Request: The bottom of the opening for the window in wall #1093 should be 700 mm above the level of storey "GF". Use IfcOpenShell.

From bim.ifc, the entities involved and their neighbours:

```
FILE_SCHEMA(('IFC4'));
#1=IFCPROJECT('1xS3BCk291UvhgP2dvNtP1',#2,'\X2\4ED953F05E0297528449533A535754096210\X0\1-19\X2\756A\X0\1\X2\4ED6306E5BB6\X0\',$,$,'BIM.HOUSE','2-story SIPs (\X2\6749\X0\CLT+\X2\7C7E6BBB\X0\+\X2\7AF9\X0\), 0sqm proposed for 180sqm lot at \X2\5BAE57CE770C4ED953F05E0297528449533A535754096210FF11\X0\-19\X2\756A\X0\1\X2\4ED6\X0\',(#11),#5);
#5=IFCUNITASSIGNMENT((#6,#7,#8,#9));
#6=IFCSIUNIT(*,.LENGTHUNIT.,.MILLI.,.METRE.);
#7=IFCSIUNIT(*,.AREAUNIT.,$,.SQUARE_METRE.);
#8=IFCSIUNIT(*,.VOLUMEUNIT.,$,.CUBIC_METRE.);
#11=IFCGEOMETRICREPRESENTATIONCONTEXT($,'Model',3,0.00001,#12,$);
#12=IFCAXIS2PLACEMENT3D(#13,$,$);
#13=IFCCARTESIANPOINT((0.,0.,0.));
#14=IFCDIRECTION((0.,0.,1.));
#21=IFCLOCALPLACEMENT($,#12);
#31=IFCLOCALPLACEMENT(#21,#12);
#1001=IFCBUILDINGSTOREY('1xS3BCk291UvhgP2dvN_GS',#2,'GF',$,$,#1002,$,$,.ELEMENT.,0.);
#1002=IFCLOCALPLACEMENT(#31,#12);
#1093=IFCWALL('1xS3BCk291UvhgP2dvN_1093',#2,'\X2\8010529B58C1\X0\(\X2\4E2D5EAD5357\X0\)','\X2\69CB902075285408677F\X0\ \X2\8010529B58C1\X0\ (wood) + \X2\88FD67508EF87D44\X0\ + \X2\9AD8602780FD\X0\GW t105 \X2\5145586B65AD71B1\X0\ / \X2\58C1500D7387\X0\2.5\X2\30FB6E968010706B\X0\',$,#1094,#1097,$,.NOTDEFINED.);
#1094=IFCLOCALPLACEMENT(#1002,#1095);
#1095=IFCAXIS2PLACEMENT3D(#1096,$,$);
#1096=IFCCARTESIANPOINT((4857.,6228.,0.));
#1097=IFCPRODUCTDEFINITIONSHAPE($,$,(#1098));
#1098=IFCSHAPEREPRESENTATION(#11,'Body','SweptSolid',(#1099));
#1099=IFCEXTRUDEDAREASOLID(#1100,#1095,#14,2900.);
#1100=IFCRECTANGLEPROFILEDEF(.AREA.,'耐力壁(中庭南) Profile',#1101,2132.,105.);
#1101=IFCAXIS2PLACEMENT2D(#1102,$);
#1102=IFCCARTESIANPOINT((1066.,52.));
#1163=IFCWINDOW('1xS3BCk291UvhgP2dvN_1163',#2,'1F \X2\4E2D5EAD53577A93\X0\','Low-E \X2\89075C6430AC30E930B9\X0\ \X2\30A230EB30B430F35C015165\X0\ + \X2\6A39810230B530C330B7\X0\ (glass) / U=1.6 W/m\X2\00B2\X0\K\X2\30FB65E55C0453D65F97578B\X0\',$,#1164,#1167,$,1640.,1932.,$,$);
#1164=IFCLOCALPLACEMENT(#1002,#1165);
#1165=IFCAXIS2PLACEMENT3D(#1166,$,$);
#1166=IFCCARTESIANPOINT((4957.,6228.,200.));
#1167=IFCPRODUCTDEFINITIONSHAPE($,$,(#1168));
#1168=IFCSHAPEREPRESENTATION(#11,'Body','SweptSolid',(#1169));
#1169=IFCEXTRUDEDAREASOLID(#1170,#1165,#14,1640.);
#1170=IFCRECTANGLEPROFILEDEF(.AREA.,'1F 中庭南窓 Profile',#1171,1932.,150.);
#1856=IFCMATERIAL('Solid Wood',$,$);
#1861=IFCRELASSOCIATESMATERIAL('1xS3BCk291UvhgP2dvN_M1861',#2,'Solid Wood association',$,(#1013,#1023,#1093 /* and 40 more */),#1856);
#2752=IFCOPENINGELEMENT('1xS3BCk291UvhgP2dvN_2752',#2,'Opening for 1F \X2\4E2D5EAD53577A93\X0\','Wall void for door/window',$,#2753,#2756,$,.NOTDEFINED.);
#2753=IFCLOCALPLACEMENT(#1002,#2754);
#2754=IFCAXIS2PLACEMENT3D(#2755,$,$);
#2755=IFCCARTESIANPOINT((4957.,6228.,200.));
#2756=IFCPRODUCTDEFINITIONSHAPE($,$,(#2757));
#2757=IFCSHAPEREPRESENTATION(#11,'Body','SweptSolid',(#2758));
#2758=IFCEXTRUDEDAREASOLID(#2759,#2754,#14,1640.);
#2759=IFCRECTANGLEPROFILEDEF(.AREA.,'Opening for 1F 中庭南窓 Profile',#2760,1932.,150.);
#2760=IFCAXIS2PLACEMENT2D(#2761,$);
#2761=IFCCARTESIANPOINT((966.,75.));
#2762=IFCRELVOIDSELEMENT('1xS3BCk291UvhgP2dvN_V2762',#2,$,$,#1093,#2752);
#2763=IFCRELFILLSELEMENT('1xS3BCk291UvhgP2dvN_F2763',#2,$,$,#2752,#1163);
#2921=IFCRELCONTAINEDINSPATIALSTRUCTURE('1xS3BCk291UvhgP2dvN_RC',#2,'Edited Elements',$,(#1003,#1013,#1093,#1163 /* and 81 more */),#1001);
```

```python
import numpy as np
import ifcopenshell
import ifcopenshell.api.geometry
import ifcopenshell.geom
import ifcopenshell.util.element
import ifcopenshell.util.placement
import ifcopenshell.util.shape
import ifcopenshell.util.unit

model = ifcopenshell.open("bim.ifc")
unit_scale = ifcopenshell.util.unit.calculate_unit_scale(model)

window = model.by_id(1163)
opening = window.FillsVoids[0].RelatingOpeningElement
storey = ifcopenshell.util.element.get_container(window, ifc_class="IfcBuildingStorey")
level = ifcopenshell.util.placement.get_local_placement(storey.ObjectPlacement)[2, 3]

# The opening's origin need not be at the sill, so measure its lowest point.
shape = ifcopenshell.geom.create_shape(ifcopenshell.geom.settings(), opening)
bottom = ifcopenshell.util.shape.get_shape_bottom_elevation(shape, shape.geometry) / unit_scale
dz = level + 0.7 / unit_scale - bottom

shift = np.array([0.0, 0.0, dz])
# The window is not placed relative to its opening, so move both.
for product in (opening, window):
    matrix = ifcopenshell.util.placement.get_local_placement(product.ObjectPlacement)
    matrix[:3, 3] += shift
    ifcopenshell.api.geometry.edit_object_placement(model, product=product, matrix=matrix, is_si=False)

print(f"moved by {dz * unit_scale:+.3f} m")

model.write("bim-out.ifc")
```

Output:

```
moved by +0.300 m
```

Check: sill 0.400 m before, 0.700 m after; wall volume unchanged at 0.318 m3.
